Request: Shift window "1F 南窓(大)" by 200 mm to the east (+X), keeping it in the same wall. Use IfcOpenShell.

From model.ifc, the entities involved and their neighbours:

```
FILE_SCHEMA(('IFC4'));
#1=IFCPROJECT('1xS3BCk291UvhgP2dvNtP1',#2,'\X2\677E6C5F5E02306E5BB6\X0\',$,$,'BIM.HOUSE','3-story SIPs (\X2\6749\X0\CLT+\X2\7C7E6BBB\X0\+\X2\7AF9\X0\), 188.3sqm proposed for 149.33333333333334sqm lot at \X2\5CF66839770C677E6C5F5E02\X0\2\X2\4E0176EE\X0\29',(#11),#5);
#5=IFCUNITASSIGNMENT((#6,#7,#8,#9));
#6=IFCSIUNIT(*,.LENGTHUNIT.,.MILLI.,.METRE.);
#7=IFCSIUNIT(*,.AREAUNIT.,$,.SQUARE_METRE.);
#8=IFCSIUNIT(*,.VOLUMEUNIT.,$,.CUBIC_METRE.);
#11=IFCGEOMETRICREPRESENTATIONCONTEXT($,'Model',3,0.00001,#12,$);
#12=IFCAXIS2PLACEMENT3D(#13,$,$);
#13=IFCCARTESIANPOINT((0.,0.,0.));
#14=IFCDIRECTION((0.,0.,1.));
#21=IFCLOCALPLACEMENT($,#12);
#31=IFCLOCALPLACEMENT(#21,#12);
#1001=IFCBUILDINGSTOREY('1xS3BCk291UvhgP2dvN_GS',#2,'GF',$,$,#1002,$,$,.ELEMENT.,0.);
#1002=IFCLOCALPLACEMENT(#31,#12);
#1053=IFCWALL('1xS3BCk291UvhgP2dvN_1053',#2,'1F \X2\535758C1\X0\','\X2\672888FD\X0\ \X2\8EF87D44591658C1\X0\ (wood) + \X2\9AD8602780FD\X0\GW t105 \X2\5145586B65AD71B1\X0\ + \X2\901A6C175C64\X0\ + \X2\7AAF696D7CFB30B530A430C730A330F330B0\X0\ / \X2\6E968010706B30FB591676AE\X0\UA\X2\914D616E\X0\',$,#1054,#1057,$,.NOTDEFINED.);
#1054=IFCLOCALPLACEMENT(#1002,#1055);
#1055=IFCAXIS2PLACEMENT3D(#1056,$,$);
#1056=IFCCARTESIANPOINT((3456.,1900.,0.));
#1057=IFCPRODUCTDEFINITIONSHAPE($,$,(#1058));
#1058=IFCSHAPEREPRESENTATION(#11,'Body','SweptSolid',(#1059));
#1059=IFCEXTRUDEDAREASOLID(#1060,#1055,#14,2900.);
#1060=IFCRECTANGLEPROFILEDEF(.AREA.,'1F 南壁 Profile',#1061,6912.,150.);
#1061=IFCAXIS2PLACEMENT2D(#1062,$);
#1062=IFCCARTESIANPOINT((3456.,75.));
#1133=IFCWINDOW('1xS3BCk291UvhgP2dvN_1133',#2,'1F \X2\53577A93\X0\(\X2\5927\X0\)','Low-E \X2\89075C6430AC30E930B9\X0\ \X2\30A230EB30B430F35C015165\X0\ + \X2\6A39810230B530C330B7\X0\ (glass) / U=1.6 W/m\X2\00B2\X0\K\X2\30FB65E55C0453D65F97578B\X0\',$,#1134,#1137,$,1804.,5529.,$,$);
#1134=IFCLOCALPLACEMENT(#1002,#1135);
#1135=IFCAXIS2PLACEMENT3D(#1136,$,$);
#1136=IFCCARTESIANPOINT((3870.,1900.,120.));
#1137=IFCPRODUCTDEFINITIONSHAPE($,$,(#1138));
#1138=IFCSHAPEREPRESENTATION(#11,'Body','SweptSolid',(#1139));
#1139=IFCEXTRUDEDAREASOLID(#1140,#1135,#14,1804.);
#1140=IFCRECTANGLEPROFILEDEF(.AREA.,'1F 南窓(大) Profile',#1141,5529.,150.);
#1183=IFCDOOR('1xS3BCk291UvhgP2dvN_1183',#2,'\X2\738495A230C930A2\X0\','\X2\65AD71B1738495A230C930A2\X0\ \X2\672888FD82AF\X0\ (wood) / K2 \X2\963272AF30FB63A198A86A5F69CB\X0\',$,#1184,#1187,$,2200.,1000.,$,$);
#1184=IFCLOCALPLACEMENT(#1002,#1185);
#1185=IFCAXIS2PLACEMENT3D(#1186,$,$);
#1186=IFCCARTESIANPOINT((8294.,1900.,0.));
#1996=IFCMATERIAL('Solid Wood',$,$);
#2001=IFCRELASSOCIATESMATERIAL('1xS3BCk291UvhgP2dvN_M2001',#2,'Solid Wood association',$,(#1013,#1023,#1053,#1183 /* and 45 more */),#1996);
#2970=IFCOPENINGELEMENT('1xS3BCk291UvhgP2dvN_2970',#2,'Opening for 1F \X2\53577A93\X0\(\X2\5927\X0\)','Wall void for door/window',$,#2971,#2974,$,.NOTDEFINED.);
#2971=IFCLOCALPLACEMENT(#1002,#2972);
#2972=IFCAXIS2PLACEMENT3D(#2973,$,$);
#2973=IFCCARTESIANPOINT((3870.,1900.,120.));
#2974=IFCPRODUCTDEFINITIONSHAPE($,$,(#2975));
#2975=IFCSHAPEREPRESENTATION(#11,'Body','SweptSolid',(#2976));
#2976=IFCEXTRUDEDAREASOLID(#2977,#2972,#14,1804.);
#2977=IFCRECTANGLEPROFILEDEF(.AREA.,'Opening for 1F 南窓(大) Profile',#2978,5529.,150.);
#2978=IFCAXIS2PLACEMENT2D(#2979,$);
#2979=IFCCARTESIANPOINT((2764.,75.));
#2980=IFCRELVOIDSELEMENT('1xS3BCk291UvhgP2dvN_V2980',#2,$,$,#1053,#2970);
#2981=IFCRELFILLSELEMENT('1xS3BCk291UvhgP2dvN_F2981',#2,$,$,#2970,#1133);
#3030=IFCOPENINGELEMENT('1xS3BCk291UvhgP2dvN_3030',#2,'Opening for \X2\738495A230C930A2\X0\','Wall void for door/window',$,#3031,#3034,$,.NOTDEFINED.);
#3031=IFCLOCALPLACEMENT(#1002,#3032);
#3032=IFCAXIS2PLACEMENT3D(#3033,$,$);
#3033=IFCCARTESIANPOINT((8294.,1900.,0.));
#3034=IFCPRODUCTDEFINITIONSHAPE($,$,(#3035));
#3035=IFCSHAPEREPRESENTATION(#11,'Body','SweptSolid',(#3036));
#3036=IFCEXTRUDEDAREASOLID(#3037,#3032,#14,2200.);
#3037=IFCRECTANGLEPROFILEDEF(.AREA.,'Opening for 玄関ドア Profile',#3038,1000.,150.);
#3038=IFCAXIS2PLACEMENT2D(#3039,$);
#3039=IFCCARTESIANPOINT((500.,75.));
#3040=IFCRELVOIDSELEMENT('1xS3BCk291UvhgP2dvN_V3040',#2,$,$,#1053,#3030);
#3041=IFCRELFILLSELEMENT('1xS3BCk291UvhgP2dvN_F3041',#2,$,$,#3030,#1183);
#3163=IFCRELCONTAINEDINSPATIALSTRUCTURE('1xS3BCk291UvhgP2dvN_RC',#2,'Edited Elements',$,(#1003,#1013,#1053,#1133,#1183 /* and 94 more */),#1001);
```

```python
import ifcopenshell
import ifcopenshell.api.geometry
import ifcopenshell.util.placement
import ifcopenshell.util.unit

model = ifcopenshell.open("model.ifc")
unit_scale = ifcopenshell.util.unit.calculate_unit_scale(model)

window = model.by_guid("1xS3BCk291UvhgP2dvN_1133")
opening = window.FillsVoids[0].RelatingOpeningElement
wall = opening.VoidsElements[0].RelatingBuildingElement

wall_matrix = ifcopenshell.util.placement.get_local_placement(wall.ObjectPlacement)
shift = wall_matrix[:3, 0] * 0.2 / unit_scale
before = ifcopenshell.util.placement.get_local_placement(window.ObjectPlacement)[:3, 3].copy()

# The window is not placed relative to its opening, so move both.
for product in (opening, window):
    matrix = ifcopenshell.util.placement.get_local_placement(product.ObjectPlacement)
    matrix[:3, 3] += shift
    ifcopenshell.api.geometry.edit_object_placement(model, product=product, matrix=matrix, is_si=False)

after = ifcopenshell.util.placement.get_local_placement(window.ObjectPlacement)[:3, 3]
print("window moved by", (after - before).round(3) + 0.0)

model.write("model-out.ifc")
```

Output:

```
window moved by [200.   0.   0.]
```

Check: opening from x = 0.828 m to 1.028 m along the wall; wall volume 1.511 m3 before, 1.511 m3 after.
